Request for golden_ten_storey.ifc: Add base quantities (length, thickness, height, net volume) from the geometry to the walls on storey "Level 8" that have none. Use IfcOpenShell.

First a look at what the model holds.

```python
import ifcopenshell
import ifcopenshell.util.element
import ifcopenshell.util.unit

model = ifcopenshell.open("golden_ten_storey.ifc")
print(model.schema)
for unit_type in ("LENGTHUNIT", "AREAUNIT", "VOLUMEUNIT"):
    print(unit_type, ifcopenshell.util.unit.calculate_unit_scale(model, unit_type))
storey = next(s for s in model.by_type("IfcBuildingStorey") if s.Name == "Level 8")
walls = [e for e in ifcopenshell.util.element.get_decomposition(storey) if e.is_a("IfcWall")]
for e in sorted(walls, key=lambda e: e.id()):
    print(e.id(), e.is_a(), e.Name, list(ifcopenshell.util.element.get_psets(e, qtos_only=True)), sep=" | ")
```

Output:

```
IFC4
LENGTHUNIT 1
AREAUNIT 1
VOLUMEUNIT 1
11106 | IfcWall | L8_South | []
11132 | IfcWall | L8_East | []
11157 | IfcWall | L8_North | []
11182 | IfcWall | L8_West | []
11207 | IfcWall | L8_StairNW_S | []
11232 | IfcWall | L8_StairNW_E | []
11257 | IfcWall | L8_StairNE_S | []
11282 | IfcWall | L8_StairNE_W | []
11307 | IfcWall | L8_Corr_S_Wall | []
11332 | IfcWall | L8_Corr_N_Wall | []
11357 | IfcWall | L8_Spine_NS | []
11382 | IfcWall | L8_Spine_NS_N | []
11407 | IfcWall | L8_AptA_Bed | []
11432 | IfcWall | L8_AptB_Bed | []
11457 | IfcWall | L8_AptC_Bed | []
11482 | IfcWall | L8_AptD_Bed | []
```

```python
import ifcopenshell
import ifcopenshell.api.pset
import ifcopenshell.geom
import ifcopenshell.util.element
import ifcopenshell.util.shape
import ifcopenshell.util.unit

model = ifcopenshell.open("golden_ten_storey.ifc")
unit_scale = ifcopenshell.util.unit.calculate_unit_scale(model)
volume_scale = ifcopenshell.util.unit.calculate_unit_scale(model, "VOLUMEUNIT")
settings = ifcopenshell.geom.settings()

storey = next(s for s in model.by_type("IfcBuildingStorey") if s.Name == "Level 8")
walls = [e for e in ifcopenshell.util.element.get_decomposition(storey) if e.is_a("IfcWall")]

for e in sorted(walls, key=lambda e: e.id()):
    if ifcopenshell.util.element.get_psets(e, qtos_only=True, should_inherit=False):
        continue
    # Geometry comes back in metres, in the element's own axes.
    shape = ifcopenshell.geom.create_shape(settings, e)
    values = {
        "Length": ifcopenshell.util.shape.get_x(shape.geometry) / unit_scale,
        "Width": ifcopenshell.util.shape.get_y(shape.geometry) / unit_scale,
        "Height": ifcopenshell.util.shape.get_z(shape.geometry) / unit_scale,
        "NetVolume": ifcopenshell.util.shape.get_volume(shape.geometry) / volume_scale,
    }
    qto = ifcopenshell.api.pset.add_qto(model, product=e, name="Qto_WallBaseQuantities")
    ifcopenshell.api.pset.edit_qto(model, qto=qto, properties=values)
    print(e.id(), {k: round(v, 3) for k, v in values.items()})

model.write("golden_ten_storey_v2.ifc")
```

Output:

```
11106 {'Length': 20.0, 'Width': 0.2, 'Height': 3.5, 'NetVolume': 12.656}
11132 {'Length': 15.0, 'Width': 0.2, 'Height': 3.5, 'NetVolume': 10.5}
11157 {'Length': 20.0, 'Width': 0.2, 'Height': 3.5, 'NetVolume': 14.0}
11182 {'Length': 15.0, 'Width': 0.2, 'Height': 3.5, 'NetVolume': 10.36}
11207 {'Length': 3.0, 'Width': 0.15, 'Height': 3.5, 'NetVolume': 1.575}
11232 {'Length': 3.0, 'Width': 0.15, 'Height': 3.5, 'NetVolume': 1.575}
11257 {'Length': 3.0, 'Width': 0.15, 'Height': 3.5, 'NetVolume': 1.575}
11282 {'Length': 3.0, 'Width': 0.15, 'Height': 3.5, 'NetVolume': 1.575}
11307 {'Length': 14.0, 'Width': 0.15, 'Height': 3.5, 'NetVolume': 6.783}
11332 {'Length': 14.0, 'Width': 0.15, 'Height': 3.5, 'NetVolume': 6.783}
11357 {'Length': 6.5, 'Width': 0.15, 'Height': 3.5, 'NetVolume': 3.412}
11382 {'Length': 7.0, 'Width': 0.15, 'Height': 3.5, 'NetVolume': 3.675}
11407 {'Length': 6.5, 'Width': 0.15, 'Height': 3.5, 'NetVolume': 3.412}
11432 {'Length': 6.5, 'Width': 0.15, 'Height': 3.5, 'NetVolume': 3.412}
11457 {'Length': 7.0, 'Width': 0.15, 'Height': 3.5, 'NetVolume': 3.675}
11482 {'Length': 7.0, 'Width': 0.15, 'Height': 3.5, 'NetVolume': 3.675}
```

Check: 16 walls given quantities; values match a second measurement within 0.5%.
